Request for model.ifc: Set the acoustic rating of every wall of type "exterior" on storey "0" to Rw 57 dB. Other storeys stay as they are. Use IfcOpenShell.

First a look at what the model holds.

```python
import ifcopenshell
import ifcopenshell.util.element

model = ifcopenshell.open("model.ifc")
print(model.schema)
storey = next(s for s in model.by_type("IfcBuildingStorey") if s.Name == "0")
walls = [e for e in ifcopenshell.util.element.get_decomposition(storey) if e.is_a("IfcWall")]
seen = {}
for e in walls:
    element_type = ifcopenshell.util.element.get_type(e)
    key = (element_type.Name if element_type != e and element_type else None, ifcopenshell.util.element.get_pset(e, "Pset_WallCommon", "AcousticRating"))
    seen[key] = seen.get(key, 0) + 1
for (name, value), count in sorted(seen.items(), key=str):
    print(count, "x", name, "|", value)
```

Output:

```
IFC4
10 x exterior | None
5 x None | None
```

```python
import ifcopenshell
import ifcopenshell.api.pset
import ifcopenshell.util.element

model = ifcopenshell.open("model.ifc")

storey = next(s for s in model.by_type("IfcBuildingStorey") if s.Name == "0")
walls = [e for e in ifcopenshell.util.element.get_decomposition(storey) if e.is_a("IfcWall")]

count = 0
for e in walls:
    element_type = ifcopenshell.util.element.get_type(e)
    if element_type in (None, e) or element_type.Name != "exterior":
        continue
    # add_pset returns the element's existing set when there is one.
    pset = ifcopenshell.api.pset.add_pset(model, product=e, name="Pset_WallCommon")
    ifcopenshell.api.pset.edit_pset(model, pset=pset, properties={"AcousticRating": "Rw 57 dB"})
    count += 1

print(count, "walls updated")

model.write("model_edited.ifc")
```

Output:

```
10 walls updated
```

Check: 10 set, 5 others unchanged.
